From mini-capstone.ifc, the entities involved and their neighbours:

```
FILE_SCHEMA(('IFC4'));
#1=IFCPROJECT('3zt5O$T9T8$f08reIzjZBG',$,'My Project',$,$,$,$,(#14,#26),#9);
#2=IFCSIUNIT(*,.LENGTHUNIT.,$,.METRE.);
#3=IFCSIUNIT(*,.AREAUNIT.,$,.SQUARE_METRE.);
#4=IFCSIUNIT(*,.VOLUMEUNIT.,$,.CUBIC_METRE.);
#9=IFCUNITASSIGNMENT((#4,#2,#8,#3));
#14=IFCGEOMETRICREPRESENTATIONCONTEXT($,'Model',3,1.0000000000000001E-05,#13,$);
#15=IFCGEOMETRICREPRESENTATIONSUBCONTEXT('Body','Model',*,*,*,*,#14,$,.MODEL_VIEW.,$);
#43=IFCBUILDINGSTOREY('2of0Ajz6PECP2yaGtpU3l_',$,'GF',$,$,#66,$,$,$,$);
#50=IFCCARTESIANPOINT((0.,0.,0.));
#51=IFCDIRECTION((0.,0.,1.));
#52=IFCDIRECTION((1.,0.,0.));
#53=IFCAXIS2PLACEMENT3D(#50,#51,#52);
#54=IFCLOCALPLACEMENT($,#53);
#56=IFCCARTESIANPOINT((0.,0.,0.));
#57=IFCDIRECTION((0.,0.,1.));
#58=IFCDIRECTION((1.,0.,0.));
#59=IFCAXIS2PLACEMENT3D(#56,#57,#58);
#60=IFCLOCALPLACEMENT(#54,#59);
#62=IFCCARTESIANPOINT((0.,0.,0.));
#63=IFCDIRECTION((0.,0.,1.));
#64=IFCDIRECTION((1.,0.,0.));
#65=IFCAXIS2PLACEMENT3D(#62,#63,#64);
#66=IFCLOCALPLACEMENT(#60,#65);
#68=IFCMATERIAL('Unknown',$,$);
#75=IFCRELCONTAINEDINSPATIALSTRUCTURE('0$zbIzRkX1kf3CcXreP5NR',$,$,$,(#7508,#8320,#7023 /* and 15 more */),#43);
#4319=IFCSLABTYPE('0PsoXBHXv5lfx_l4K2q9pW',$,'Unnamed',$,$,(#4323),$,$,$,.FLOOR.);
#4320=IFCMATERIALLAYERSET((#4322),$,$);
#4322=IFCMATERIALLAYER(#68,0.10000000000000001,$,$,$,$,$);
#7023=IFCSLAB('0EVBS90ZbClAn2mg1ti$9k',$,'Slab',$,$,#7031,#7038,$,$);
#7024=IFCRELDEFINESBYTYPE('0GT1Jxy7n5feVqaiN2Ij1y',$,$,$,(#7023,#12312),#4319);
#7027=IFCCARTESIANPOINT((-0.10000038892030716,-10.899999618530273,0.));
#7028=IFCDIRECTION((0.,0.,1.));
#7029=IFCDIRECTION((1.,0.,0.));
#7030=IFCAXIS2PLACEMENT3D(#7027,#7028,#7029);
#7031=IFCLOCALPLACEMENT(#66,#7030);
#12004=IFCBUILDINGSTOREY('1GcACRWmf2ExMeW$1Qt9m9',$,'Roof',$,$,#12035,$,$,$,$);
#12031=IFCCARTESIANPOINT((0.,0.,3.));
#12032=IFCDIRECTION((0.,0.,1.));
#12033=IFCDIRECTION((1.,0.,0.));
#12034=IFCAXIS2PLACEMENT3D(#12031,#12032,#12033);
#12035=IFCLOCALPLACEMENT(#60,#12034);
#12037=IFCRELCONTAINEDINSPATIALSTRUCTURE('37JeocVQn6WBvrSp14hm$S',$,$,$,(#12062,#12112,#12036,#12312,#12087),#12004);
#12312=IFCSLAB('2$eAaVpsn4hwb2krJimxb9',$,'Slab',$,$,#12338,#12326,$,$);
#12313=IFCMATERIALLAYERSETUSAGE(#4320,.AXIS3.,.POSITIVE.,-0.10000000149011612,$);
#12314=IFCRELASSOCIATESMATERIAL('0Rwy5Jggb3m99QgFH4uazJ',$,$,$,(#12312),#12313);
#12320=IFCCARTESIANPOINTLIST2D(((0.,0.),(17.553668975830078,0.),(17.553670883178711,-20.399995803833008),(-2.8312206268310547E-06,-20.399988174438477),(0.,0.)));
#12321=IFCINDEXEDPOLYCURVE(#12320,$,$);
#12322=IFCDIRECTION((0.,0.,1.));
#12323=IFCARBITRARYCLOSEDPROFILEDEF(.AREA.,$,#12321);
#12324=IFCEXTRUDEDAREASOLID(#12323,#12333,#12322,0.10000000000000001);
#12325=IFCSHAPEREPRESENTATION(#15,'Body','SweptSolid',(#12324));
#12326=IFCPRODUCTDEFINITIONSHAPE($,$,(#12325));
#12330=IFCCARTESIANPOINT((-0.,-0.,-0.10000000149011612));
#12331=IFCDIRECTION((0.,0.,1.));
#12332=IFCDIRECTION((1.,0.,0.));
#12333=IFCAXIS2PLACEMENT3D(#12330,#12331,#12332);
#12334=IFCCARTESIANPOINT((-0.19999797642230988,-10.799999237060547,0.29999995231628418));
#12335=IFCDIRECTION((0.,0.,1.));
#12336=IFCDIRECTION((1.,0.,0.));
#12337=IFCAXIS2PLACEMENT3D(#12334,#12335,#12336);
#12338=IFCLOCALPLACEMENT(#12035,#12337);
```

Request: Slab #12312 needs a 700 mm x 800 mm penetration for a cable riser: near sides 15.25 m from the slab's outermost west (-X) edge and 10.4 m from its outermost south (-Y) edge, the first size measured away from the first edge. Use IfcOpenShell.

```python
import numpy as np
import ifcopenshell
import ifcopenshell.api.feature
import ifcopenshell.api.geometry
import ifcopenshell.api.root
import ifcopenshell.geom
import ifcopenshell.util.placement
import ifcopenshell.util.representation
import ifcopenshell.util.shape
import ifcopenshell.util.unit

model = ifcopenshell.open("mini-capstone.ifc")
unit_scale = ifcopenshell.util.unit.calculate_unit_scale(model)
settings = ifcopenshell.geom.settings()


def volume(element):
    """Net volume in cubic metres, openings subtracted."""
    shape = ifcopenshell.geom.create_shape(settings, element)
    return ifcopenshell.util.shape.get_volume(shape.geometry)


slab = model.by_guid("2$eAaVpsn4hwb2krJimxb9")
before = volume(slab)

# Extent in the slab's own axes, in metres. The edges named are its -X and -Y sides.
slab_shape = ifcopenshell.geom.create_shape(settings, slab)
vertices = ifcopenshell.util.shape.get_vertices(slab_shape.geometry)
x_min, y_min, bottom = vertices.min(axis=0)
top = vertices[:, 2].max()

opening = ifcopenshell.api.root.create_entity(model, ifc_class="IfcOpeningElement", name="Cable riser opening", predefined_type="OPENING")
context = ifcopenshell.util.representation.get_context(model, "Model", "Body", "MODEL_VIEW")
width, depth = 0.7, 0.8
outline = [(0.0, 0.0), (width, 0.0), (width, depth), (0.0, depth), (0.0, 0.0)]
# Overshoot both faces by 50 mm so the cut is clean.
shape = ifcopenshell.api.geometry.add_slab_representation(
    model, context=context, depth=top - bottom + 0.1, polyline=outline
)
ifcopenshell.api.geometry.assign_representation(model, product=opening, representation=shape)

matrix = ifcopenshell.util.placement.get_local_placement(slab.ObjectPlacement)
matrix[:, 3] = matrix @ np.append(np.array([x_min + 15.25, y_min + 10.4, bottom - 0.05]) / unit_scale, 1.0)
ifcopenshell.api.geometry.edit_object_placement(model, product=opening, matrix=matrix, is_si=False)
ifcopenshell.api.feature.add_feature(model, feature=opening, element=slab)

after = volume(slab)

print(f"slab volume {before:.3f} -> {after:.3f} m3")

model.write("mini-capstone_rev.ifc")
```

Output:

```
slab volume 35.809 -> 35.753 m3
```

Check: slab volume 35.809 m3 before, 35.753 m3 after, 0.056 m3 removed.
